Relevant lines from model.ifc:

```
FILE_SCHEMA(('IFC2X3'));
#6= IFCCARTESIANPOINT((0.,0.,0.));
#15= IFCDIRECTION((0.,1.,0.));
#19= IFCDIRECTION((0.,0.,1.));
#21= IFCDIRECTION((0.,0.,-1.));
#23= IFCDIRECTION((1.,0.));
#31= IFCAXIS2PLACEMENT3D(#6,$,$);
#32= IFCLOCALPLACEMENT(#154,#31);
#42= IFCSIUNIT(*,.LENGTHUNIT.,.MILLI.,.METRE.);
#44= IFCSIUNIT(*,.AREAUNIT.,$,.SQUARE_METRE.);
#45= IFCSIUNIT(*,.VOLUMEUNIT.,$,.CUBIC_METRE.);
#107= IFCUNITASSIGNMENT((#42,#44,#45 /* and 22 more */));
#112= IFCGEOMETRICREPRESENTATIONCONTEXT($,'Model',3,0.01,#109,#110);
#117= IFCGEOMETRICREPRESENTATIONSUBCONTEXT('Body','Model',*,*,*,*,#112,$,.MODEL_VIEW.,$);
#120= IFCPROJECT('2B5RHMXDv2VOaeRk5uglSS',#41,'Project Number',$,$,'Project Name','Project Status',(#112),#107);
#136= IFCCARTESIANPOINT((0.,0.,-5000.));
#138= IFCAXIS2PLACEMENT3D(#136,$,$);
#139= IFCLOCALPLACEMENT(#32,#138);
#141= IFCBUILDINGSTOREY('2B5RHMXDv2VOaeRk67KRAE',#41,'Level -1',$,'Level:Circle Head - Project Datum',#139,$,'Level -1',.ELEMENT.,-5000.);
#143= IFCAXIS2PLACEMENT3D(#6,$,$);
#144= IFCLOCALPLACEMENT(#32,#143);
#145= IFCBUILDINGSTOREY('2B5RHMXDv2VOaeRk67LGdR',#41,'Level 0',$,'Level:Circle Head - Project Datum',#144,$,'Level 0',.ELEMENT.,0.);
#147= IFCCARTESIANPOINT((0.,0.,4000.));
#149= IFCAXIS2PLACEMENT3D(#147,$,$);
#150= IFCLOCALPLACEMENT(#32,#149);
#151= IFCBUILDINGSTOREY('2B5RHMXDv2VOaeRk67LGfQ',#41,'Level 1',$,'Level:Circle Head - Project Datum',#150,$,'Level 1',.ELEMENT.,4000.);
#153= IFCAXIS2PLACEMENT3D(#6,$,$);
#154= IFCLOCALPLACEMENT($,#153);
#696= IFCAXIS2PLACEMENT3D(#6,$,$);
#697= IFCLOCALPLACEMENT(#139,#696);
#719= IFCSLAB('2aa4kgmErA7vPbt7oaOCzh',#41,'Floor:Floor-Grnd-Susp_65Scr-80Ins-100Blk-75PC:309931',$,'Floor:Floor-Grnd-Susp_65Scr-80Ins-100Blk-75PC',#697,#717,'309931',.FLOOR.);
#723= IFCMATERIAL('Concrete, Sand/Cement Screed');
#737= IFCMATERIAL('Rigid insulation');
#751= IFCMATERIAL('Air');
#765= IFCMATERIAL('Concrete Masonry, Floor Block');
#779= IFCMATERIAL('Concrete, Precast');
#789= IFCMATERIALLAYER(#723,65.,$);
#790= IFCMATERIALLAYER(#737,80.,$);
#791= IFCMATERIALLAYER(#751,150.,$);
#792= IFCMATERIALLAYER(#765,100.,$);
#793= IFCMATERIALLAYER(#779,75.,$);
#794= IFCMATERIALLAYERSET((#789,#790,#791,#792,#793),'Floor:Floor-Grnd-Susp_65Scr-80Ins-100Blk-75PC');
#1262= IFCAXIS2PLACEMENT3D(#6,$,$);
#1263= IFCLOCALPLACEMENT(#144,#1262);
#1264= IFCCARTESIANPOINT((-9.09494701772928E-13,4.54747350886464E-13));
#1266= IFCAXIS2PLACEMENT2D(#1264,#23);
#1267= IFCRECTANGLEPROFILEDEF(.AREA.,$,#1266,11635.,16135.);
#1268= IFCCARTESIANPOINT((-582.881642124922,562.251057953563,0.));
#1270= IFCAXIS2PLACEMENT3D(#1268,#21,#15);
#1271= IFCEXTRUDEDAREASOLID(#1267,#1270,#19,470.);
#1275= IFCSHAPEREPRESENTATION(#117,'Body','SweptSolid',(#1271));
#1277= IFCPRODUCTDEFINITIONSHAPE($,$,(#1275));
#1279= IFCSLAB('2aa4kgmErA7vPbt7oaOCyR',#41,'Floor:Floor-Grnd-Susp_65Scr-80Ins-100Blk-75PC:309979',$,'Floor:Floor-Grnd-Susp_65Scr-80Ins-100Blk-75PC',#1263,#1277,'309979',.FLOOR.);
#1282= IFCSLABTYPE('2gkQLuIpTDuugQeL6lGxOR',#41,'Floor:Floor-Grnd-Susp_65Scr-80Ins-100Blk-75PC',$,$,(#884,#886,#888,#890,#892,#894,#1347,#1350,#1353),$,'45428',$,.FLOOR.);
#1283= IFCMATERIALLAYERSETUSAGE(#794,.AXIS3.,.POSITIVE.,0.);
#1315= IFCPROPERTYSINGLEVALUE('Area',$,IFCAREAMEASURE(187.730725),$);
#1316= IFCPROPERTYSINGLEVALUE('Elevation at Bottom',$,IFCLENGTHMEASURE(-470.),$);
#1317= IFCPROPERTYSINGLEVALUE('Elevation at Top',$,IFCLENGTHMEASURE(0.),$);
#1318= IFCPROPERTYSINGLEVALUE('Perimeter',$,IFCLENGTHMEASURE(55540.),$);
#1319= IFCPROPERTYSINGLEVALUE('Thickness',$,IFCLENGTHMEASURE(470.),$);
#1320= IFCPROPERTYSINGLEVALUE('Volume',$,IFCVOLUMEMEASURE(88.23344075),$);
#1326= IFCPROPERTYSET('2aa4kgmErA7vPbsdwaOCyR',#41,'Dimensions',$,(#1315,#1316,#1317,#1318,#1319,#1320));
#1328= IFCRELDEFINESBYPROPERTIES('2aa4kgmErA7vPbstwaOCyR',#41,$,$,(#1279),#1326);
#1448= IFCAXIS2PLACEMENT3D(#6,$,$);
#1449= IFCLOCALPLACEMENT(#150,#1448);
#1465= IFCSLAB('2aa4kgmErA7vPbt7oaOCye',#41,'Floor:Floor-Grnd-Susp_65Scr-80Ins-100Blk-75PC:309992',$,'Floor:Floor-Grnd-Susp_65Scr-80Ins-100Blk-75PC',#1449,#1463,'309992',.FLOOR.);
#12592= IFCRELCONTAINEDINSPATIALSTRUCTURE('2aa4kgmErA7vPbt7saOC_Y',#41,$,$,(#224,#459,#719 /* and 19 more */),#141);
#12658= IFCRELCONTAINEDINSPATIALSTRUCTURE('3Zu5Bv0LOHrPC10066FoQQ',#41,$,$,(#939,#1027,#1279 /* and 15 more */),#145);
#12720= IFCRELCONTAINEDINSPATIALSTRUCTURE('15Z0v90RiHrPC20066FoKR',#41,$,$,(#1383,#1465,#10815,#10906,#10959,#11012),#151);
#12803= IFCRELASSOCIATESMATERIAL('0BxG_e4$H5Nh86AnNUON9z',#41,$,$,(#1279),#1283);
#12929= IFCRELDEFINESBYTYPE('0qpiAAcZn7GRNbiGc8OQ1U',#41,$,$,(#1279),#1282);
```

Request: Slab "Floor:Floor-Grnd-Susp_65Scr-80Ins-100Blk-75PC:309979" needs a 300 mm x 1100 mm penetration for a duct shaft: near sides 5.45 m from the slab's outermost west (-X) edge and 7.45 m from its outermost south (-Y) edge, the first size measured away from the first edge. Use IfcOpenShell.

```python
import numpy as np
import ifcopenshell
import ifcopenshell.api.feature
import ifcopenshell.api.geometry
import ifcopenshell.api.pset
import ifcopenshell.api.root
import ifcopenshell.geom
import ifcopenshell.util.element
import ifcopenshell.util.placement
import ifcopenshell.util.representation
import ifcopenshell.util.shape
import ifcopenshell.util.unit

model = ifcopenshell.open("model.ifc")
unit_scale = ifcopenshell.util.unit.calculate_unit_scale(model)
area_scale = ifcopenshell.util.unit.calculate_unit_scale(model, "AREAUNIT")
volume_scale = ifcopenshell.util.unit.calculate_unit_scale(model, "VOLUMEUNIT")
settings = ifcopenshell.geom.settings()


def volume(element):
    """Net volume in cubic metres, openings subtracted."""
    shape = ifcopenshell.geom.create_shape(settings, element)
    return ifcopenshell.util.shape.get_volume(shape.geometry)


slab = model.by_guid("2aa4kgmErA7vPbt7oaOCyR")
before = volume(slab)

# Extent in the slab's own axes, in metres. The edges named are its -X and -Y sides.
slab_shape = ifcopenshell.geom.create_shape(settings, slab)
vertices = ifcopenshell.util.shape.get_vertices(slab_shape.geometry)
x_min, y_min, bottom = vertices.min(axis=0)
top = vertices[:, 2].max()

opening = ifcopenshell.api.root.create_entity(model, ifc_class="IfcOpeningElement", name="Duct shaft opening")
context = ifcopenshell.util.representation.get_context(model, "Model", "Body", "MODEL_VIEW")
width, depth = 0.3, 1.1
outline = [(0.0, 0.0), (width, 0.0), (width, depth), (0.0, depth), (0.0, 0.0)]
# Overshoot both faces by 50 mm so the cut is clean.
shape = ifcopenshell.api.geometry.add_slab_representation(
    model, context=context, depth=top - bottom + 0.1, polyline=outline
)
ifcopenshell.api.geometry.assign_representation(model, product=opening, representation=shape)

matrix = ifcopenshell.util.placement.get_local_placement(slab.ObjectPlacement)
matrix[:, 3] = matrix @ np.append(np.array([x_min + 5.45, y_min + 7.45, bottom - 0.05]) / unit_scale, 1.0)
ifcopenshell.api.geometry.edit_object_placement(model, product=opening, matrix=matrix, is_si=False)
ifcopenshell.api.feature.add_feature(model, feature=opening, element=slab)

after = volume(slab)

# Update the slab's stored quantities.
pset = model.by_id(ifcopenshell.util.element.get_pset(slab, "Dimensions", should_inherit=False)["id"])
ifcopenshell.api.pset.edit_pset(model, pset=pset, properties={
    "Area": model.create_entity("IfcAreaMeasure", after / (top - bottom) / area_scale),
    "Volume": model.create_entity("IfcVolumeMeasure", after / volume_scale),
})

print(f"slab volume {before:.3f} -> {after:.3f} m3")

model.write("model_updated.ifc")
```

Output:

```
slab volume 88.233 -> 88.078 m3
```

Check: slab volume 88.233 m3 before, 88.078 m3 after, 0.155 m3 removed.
